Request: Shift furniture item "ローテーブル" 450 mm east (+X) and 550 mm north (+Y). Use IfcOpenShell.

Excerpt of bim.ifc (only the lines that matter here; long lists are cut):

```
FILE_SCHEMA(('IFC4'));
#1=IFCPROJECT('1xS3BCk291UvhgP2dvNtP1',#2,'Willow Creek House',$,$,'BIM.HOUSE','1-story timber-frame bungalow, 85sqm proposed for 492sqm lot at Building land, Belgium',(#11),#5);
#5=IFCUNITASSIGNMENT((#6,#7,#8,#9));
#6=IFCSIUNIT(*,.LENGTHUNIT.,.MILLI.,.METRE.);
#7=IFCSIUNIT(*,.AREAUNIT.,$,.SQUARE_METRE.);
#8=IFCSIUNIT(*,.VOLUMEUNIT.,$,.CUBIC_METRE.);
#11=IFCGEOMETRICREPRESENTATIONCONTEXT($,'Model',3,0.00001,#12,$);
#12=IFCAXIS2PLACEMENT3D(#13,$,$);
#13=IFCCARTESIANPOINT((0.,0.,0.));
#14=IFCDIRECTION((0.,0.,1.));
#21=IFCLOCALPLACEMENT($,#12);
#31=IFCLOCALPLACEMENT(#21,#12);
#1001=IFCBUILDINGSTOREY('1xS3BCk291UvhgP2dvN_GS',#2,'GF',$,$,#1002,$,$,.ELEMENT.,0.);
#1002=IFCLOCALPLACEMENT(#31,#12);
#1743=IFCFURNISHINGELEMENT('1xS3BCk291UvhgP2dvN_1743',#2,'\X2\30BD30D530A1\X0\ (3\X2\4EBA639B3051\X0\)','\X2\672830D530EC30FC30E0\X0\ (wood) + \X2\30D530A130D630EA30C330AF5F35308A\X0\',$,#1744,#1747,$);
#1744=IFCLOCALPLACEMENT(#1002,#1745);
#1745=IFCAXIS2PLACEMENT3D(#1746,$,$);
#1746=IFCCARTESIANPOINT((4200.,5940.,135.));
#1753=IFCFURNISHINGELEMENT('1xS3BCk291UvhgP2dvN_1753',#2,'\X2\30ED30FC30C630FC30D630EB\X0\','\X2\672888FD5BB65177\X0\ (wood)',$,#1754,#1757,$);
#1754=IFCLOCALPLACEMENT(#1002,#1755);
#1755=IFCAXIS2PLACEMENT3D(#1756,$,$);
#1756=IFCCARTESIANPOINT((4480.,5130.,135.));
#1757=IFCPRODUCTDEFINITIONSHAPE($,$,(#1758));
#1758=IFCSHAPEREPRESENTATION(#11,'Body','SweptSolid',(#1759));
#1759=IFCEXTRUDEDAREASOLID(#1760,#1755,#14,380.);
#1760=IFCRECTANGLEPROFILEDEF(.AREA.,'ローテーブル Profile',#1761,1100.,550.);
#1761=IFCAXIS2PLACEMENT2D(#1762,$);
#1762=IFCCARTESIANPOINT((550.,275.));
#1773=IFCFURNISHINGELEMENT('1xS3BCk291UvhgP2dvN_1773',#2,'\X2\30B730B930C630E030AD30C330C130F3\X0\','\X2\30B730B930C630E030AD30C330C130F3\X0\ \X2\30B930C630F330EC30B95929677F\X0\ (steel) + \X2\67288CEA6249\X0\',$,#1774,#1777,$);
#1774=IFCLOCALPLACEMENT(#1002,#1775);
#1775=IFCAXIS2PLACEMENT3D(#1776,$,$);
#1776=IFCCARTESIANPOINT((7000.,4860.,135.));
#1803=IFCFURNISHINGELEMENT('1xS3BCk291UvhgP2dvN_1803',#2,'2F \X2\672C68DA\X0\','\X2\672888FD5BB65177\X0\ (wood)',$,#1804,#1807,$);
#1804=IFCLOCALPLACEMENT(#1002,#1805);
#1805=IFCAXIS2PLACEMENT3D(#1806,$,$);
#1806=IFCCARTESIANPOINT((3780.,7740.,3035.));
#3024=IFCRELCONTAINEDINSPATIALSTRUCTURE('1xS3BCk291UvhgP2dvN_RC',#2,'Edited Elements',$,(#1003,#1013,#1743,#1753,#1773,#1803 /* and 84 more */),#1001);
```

```python
import ifcopenshell
import ifcopenshell.api.geometry
import ifcopenshell.util.placement

model = ifcopenshell.open("bim.ifc")

item = model.by_guid("1xS3BCk291UvhgP2dvN_1753")
matrix = ifcopenshell.util.placement.get_local_placement(item.ObjectPlacement)
matrix[0, 3] += 450.0
matrix[1, 3] += 550.0
ifcopenshell.api.geometry.edit_object_placement(model, product=item, matrix=matrix, is_si=False)

print(ifcopenshell.util.placement.get_local_placement(item.ObjectPlacement).round(3) + 0.0)

model.write("bim-out.ifc")
```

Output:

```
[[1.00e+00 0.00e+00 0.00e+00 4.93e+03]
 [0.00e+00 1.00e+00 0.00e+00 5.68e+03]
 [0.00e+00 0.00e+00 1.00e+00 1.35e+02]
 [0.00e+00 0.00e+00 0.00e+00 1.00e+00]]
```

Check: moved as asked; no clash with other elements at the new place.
